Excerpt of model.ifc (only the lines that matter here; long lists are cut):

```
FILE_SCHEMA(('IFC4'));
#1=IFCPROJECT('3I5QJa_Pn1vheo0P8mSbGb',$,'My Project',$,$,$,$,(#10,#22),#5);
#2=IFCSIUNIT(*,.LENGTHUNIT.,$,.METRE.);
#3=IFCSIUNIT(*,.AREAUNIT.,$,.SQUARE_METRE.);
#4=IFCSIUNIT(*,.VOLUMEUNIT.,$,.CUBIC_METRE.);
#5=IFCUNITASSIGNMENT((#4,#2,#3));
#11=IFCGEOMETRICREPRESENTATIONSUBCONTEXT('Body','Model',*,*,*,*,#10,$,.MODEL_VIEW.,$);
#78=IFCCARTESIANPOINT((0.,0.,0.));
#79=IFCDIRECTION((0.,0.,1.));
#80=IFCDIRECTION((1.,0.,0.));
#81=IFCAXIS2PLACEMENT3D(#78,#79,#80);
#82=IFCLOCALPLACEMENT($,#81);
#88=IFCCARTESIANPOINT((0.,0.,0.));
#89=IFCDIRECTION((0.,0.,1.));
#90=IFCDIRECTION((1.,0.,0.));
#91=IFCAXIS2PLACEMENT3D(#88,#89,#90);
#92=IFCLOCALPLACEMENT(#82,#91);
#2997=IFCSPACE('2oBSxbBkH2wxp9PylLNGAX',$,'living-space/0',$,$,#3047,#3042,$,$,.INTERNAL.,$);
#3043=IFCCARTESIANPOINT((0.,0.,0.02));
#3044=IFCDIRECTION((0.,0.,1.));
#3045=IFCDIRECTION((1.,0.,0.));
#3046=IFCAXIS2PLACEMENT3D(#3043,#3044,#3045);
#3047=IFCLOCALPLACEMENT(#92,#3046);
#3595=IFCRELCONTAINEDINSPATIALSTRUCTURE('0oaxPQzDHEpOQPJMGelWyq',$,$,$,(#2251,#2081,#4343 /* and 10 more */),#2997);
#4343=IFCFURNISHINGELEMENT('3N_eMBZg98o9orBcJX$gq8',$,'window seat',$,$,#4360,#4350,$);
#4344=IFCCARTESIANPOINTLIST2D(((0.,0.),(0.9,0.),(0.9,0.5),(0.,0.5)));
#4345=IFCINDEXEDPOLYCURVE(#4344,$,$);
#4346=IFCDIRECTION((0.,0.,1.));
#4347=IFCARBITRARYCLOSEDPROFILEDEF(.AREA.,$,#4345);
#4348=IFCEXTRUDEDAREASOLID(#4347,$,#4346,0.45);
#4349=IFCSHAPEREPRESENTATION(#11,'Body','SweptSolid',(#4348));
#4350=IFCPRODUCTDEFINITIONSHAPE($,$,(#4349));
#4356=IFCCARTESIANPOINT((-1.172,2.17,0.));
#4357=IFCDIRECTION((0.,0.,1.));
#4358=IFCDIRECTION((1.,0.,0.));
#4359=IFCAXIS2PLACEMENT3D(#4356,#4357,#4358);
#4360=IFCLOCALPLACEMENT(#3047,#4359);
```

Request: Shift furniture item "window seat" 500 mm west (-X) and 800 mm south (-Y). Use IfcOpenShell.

```python
import ifcopenshell
import ifcopenshell.api.geometry
import ifcopenshell.util.placement
import ifcopenshell.util.unit

model = ifcopenshell.open("model.ifc")
unit_scale = ifcopenshell.util.unit.calculate_unit_scale(model)

item = model.by_id(4343)
matrix = ifcopenshell.util.placement.get_local_placement(item.ObjectPlacement)
matrix[0, 3] -= 0.5 / unit_scale
matrix[1, 3] -= 0.8 / unit_scale
ifcopenshell.api.geometry.edit_object_placement(model, product=item, matrix=matrix, is_si=False)

print(ifcopenshell.util.placement.get_local_placement(item.ObjectPlacement).round(3) + 0.0)

model.write("model_v2.ifc")
```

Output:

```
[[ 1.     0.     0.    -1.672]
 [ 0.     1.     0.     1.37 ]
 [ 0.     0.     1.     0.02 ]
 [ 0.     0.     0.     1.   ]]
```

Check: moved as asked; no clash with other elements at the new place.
